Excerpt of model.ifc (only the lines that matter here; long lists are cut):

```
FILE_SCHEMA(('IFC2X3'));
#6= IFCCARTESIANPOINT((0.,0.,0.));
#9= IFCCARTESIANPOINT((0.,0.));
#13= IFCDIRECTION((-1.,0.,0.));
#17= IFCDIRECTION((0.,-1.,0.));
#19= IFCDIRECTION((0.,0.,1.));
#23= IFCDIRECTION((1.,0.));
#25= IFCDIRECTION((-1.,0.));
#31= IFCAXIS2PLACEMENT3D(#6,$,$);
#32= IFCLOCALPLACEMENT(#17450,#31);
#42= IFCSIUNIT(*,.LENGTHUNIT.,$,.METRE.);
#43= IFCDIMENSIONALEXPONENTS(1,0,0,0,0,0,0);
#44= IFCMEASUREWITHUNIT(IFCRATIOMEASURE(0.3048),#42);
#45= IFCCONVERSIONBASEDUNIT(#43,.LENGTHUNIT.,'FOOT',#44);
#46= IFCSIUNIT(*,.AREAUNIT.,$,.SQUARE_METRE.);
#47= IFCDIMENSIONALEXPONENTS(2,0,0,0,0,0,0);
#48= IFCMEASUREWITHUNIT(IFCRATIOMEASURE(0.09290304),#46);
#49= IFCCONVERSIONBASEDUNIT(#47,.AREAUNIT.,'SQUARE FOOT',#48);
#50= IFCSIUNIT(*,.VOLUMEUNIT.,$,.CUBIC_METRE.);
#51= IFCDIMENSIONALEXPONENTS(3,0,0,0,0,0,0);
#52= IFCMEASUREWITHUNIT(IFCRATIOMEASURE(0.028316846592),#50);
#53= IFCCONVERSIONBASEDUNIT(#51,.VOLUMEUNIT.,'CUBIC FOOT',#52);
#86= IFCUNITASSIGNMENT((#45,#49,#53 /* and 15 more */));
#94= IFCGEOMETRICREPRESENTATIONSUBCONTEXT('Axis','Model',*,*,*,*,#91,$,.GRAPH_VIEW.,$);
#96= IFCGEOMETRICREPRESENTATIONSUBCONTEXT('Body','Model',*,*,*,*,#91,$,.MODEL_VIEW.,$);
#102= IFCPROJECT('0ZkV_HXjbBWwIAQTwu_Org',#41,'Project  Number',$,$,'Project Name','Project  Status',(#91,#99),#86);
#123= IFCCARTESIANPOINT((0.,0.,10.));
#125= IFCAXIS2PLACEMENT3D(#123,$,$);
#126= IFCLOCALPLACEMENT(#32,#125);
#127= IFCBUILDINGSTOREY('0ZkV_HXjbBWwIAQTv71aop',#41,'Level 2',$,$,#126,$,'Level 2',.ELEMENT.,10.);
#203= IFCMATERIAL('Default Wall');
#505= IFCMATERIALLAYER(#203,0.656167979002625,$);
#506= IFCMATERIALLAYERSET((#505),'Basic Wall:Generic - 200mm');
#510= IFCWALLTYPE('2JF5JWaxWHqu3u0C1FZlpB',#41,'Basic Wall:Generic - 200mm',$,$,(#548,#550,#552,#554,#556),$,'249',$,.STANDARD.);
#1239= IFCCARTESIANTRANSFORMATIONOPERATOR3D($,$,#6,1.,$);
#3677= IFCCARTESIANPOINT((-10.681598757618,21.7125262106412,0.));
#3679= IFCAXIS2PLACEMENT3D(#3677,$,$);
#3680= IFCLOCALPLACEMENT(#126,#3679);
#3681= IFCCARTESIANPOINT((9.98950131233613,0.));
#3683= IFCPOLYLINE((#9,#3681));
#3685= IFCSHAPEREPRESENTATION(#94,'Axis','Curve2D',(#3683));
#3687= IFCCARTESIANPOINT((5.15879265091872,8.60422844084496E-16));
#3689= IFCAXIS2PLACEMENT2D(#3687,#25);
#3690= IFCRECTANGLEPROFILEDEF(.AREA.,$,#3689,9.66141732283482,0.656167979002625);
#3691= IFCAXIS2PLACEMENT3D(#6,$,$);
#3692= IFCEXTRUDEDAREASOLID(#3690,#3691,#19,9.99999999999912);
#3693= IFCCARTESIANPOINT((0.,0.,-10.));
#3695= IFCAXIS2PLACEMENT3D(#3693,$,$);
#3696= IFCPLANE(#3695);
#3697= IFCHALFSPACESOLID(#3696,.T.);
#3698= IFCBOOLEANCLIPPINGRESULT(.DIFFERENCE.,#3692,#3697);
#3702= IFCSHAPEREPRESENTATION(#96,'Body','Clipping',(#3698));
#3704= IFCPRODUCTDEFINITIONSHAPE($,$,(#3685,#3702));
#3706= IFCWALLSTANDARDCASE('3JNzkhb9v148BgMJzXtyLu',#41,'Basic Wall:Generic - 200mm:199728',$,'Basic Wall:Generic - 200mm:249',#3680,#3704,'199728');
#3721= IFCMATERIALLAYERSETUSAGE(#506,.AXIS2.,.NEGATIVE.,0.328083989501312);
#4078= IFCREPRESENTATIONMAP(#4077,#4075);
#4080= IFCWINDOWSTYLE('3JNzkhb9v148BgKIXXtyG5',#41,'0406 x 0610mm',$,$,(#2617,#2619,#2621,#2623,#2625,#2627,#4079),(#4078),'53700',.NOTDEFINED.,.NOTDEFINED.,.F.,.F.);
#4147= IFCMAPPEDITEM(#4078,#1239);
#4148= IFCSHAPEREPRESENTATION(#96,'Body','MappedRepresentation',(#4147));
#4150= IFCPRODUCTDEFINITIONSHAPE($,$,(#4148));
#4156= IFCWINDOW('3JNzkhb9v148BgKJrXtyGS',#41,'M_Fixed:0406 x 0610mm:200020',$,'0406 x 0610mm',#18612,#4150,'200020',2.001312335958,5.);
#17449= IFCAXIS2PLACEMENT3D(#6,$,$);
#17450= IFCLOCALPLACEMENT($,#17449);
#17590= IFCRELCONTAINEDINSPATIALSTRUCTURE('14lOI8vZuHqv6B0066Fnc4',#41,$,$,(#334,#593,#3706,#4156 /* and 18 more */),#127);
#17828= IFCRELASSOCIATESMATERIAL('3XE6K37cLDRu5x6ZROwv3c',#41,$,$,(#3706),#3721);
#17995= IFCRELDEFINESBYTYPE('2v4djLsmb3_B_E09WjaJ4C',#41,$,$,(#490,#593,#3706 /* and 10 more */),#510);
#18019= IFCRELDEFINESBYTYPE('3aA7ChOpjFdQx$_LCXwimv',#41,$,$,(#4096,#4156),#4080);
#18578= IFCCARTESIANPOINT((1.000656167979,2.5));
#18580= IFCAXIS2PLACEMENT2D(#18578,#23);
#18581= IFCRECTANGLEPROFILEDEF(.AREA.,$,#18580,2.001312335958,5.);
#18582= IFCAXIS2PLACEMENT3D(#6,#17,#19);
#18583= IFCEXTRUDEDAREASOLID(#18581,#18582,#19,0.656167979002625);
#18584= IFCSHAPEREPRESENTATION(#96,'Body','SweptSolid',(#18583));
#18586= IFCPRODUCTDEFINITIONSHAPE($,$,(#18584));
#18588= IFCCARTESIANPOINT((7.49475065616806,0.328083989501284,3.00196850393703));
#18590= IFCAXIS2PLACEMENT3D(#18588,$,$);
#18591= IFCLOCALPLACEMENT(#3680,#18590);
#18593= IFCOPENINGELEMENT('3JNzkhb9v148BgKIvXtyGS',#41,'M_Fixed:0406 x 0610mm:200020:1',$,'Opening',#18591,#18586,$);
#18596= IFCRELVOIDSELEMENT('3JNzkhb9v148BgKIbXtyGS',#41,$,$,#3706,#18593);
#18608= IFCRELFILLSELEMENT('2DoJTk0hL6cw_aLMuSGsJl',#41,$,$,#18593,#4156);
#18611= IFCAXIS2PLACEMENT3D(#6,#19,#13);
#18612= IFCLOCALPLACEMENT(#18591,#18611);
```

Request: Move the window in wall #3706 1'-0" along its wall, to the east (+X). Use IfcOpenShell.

```python
import ifcopenshell
import ifcopenshell.api.geometry
import ifcopenshell.util.placement
import ifcopenshell.util.unit

model = ifcopenshell.open("model.ifc")
unit_scale = ifcopenshell.util.unit.calculate_unit_scale(model)

window = model.by_guid("3JNzkhb9v148BgKJrXtyGS")
opening = window.FillsVoids[0].RelatingOpeningElement
wall = opening.VoidsElements[0].RelatingBuildingElement

wall_matrix = ifcopenshell.util.placement.get_local_placement(wall.ObjectPlacement)
shift = wall_matrix[:3, 0] * 12 * 0.0254 / unit_scale
before = ifcopenshell.util.placement.get_local_placement(window.ObjectPlacement)[:3, 3].copy()

# The window is placed relative to its opening, so it follows when the opening moves.
matrix = ifcopenshell.util.placement.get_local_placement(opening.ObjectPlacement)
matrix[:3, 3] += shift
ifcopenshell.api.geometry.edit_object_placement(
    model, product=opening, matrix=matrix, is_si=False, should_transform_children=True
)

after = ifcopenshell.util.placement.get_local_placement(window.ObjectPlacement)[:3, 3]
print("window moved by", (after - before).round(3) + 0.0)

model.write("model_updated.ifc")
```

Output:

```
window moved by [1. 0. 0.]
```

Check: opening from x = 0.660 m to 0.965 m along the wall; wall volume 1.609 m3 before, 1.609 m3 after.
